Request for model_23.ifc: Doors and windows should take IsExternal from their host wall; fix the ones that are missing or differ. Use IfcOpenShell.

First a look at what the model holds.

```python
import ifcopenshell
import ifcopenshell.util.element

model = ifcopenshell.open("model_23.ifc")
print(model.schema)
seen = {}
for e in model.by_type("IfcDoor") + model.by_type("IfcWindow"):
    if not e.FillsVoids:
        continue
    host = e.FillsVoids[0].RelatingOpeningElement.VoidsElements[0].RelatingBuildingElement
    own = ifcopenshell.util.element.get_pset(e, f"Pset_{e.is_a()[3:].removesuffix('StandardCase')}Common", "IsExternal")
    wall = ifcopenshell.util.element.get_pset(host, "Pset_WallCommon", "IsExternal")
    seen[e.is_a(), own, wall] = seen.get((e.is_a(), own, wall), 0) + 1
for (cls, own, wall), count in sorted(seen.items(), key=str):
    print(count, cls, "IsExternal:", own, "| host wall:", wall)
```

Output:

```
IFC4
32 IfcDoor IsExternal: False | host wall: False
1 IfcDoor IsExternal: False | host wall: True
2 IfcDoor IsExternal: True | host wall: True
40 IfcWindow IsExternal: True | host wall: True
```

```python
import ifcopenshell
import ifcopenshell.api.pset
import ifcopenshell.util.element

model = ifcopenshell.open("model_23.ifc")

count = 0
for ifc_class, pset_name in (("IfcDoor", "Pset_DoorCommon"), ("IfcWindow", "Pset_WindowCommon")):
    for e in model.by_type(ifc_class):
        if not e.FillsVoids:
            continue
        host = e.FillsVoids[0].RelatingOpeningElement.VoidsElements[0].RelatingBuildingElement
        external = ifcopenshell.util.element.get_pset(host, "Pset_WallCommon", "IsExternal")
        if external is None or ifcopenshell.util.element.get_pset(e, pset_name, "IsExternal") == external:
            continue
        pset = ifcopenshell.api.pset.add_pset(model, product=e, name=pset_name)
        ifcopenshell.api.pset.edit_pset(model, pset=pset, properties={"IsExternal": external})
        count += 1

print(count, "updated")

model.write("model_23-out.ifc")
```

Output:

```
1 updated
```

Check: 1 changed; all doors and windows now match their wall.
